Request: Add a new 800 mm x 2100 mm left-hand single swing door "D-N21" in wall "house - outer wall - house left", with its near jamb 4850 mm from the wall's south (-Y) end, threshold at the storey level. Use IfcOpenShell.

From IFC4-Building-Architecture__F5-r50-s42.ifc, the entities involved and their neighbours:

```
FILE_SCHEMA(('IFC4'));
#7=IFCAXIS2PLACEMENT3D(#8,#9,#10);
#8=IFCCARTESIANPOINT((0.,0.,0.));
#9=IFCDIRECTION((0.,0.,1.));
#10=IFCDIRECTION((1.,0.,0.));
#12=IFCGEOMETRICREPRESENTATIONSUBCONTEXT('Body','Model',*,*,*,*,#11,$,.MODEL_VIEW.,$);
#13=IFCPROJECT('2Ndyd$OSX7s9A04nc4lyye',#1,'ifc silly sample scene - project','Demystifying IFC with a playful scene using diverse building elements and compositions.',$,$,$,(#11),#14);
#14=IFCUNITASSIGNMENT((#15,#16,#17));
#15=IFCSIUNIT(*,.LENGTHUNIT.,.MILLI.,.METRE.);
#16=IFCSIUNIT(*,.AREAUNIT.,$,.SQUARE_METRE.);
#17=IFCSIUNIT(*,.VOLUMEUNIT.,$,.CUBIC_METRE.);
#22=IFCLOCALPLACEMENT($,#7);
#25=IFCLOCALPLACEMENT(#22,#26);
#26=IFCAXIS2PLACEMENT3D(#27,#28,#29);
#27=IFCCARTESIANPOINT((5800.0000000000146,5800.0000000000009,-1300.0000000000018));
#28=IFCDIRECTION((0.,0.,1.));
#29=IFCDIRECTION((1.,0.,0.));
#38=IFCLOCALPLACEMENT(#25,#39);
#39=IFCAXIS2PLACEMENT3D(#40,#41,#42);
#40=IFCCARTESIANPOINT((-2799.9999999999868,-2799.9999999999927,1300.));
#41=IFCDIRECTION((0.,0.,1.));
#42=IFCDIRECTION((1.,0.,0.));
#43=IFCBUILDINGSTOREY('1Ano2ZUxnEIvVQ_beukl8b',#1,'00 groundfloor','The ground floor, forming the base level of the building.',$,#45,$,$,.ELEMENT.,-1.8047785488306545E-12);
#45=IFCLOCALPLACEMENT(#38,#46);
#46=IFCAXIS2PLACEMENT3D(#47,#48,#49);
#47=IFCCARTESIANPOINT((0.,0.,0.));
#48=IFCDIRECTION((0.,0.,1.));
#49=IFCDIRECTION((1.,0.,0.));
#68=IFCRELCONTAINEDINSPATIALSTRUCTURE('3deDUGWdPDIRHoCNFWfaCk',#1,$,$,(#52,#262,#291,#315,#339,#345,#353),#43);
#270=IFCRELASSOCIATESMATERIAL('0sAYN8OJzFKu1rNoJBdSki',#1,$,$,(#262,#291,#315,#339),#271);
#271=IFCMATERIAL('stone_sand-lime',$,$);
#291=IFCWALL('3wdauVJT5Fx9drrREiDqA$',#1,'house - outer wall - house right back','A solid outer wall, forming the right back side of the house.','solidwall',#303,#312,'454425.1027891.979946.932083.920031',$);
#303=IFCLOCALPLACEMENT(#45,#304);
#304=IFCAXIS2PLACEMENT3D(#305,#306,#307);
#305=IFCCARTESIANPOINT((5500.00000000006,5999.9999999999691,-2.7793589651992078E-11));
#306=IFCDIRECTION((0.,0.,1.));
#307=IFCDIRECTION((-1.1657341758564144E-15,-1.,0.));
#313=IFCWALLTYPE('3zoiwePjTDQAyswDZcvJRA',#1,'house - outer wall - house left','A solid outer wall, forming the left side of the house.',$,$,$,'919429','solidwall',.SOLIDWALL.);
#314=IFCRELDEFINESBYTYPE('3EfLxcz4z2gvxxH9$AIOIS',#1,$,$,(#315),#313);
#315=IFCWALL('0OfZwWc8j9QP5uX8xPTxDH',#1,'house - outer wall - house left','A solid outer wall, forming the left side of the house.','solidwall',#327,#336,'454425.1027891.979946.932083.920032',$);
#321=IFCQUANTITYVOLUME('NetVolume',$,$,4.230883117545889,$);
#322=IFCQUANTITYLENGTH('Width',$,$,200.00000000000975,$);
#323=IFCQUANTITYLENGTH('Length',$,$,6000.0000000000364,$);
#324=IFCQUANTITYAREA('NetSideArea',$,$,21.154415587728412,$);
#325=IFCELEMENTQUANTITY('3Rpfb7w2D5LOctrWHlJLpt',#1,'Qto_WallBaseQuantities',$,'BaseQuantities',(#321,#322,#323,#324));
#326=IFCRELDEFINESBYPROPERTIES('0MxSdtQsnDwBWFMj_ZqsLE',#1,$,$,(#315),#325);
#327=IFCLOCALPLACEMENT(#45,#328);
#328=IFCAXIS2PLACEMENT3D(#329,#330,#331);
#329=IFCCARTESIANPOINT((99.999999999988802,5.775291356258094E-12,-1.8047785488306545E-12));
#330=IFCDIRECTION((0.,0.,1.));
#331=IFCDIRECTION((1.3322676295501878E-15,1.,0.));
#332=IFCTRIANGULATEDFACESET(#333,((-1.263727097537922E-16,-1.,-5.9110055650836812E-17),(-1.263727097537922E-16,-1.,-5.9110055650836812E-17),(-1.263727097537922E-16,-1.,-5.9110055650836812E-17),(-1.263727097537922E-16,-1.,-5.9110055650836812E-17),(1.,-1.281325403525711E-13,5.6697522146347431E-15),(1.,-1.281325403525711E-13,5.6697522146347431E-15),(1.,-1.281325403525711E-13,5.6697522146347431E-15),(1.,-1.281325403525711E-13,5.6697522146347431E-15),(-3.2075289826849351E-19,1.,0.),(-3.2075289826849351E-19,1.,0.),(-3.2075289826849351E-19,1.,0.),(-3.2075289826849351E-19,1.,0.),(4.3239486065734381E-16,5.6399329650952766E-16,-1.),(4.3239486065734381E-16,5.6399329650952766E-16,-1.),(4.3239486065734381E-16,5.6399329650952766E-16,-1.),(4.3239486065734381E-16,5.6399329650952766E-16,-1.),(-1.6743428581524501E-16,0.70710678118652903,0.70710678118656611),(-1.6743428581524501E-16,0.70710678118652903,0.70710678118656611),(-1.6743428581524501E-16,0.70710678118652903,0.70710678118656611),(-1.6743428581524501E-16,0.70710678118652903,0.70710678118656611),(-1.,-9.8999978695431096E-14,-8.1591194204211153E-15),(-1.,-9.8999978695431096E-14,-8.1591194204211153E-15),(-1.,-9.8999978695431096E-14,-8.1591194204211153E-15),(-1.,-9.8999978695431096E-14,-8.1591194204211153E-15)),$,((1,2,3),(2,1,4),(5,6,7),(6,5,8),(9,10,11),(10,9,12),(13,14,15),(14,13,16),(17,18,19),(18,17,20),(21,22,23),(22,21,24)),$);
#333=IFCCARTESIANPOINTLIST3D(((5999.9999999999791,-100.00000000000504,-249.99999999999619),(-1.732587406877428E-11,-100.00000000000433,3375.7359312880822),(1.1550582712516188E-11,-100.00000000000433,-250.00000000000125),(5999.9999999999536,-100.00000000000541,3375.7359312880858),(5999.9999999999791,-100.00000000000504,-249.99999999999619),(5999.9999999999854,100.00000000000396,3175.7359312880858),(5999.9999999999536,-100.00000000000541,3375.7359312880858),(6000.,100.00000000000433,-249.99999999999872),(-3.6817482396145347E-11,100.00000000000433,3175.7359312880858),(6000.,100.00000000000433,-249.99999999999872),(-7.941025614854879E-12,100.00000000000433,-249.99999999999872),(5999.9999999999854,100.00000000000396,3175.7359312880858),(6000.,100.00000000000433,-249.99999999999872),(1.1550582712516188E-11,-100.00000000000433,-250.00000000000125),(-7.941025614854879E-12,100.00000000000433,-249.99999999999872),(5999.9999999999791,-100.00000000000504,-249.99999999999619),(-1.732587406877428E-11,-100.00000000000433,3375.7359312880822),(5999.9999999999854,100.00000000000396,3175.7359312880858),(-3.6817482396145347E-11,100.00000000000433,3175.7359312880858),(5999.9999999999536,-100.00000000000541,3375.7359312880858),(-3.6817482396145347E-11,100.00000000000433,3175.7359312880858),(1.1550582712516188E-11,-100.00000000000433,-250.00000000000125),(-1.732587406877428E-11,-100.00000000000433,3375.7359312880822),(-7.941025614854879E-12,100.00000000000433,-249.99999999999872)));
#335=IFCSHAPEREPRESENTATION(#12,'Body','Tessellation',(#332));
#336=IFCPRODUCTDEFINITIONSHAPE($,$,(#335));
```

```python
import numpy as np
import ifcopenshell
import ifcopenshell.api.feature
import ifcopenshell.api.geometry
import ifcopenshell.api.pset
import ifcopenshell.api.root
import ifcopenshell.api.spatial
import ifcopenshell.geom
import ifcopenshell.util.element
import ifcopenshell.util.placement
import ifcopenshell.util.representation
import ifcopenshell.util.shape
import ifcopenshell.util.unit

model = ifcopenshell.open("IFC4-Building-Architecture__F5-r50-s42.ifc")
unit_scale = ifcopenshell.util.unit.calculate_unit_scale(model)
area_scale = ifcopenshell.util.unit.calculate_unit_scale(model, "AREAUNIT")
volume_scale = ifcopenshell.util.unit.calculate_unit_scale(model, "VOLUMEUNIT")
settings = ifcopenshell.geom.settings()


def volume(element):
    """Net volume in cubic metres, openings subtracted."""
    shape = ifcopenshell.geom.create_shape(settings, element)
    return ifcopenshell.util.shape.get_volume(shape.geometry)


wall = model.by_guid("0OfZwWc8j9QP5uX8xPTxDH")
storey = ifcopenshell.util.element.get_container(wall, ifc_class="IfcBuildingStorey")
context = ifcopenshell.util.representation.get_context(model, "Model", "Body", "MODEL_VIEW")
before = volume(wall)

width, height, from_end, sill = 0.8, 2.1, 4.85, 0.0  # metres

# The wall runs along its own X axis, and the end named is its -X end.
wall_shape = ifcopenshell.geom.create_shape(settings, wall)
x, y, z = ifcopenshell.util.shape.get_vertices(wall_shape.geometry).T
start = x.min() + from_end
face, thickness = float(y.min()), float(y.max() - y.min())
wall_matrix = ifcopenshell.util.placement.get_local_placement(wall.ObjectPlacement)
level = ifcopenshell.util.placement.get_local_placement(storey.ObjectPlacement)[2, 3]


def in_wall(x, y):
    """Placement at x, y metres in the wall's axes, at sill height."""
    matrix = wall_matrix.copy()
    matrix[:, 3] = wall_matrix @ np.array([x / unit_scale, y / unit_scale, 0.0, 1.0])
    matrix[2, 3] = level + sill / unit_scale
    return matrix


# Opening: a box that overshoots both wall faces by 50 mm.
opening = ifcopenshell.api.root.create_entity(model, ifc_class="IfcOpeningElement", predefined_type="OPENING")
box = ifcopenshell.api.geometry.add_wall_representation(
    model, context=context, length=width, height=height, thickness=thickness + 0.1
)
ifcopenshell.api.geometry.assign_representation(model, product=opening, representation=box)
ifcopenshell.api.geometry.edit_object_placement(model, product=opening, matrix=in_wall(start, face - 0.05), is_si=False)
ifcopenshell.api.feature.add_feature(model, feature=opening, element=wall)

door = ifcopenshell.api.root.create_entity(model, ifc_class="IfcDoor", name="D-N21", predefined_type="DOOR")
door.OverallWidth, door.OverallHeight = width / unit_scale, height / unit_scale
door.OperationType = "SINGLE_SWING_LEFT"
body = ifcopenshell.api.geometry.add_door_representation(
    model,
    context=context,
    overall_width=door.OverallWidth,
    overall_height=door.OverallHeight,
    operation_type="SINGLE_SWING_LEFT",
    lining_properties={"LiningDepth": thickness / unit_scale, "ThresholdDepth": thickness / unit_scale},
)
ifcopenshell.api.geometry.assign_representation(model, product=door, representation=body)
ifcopenshell.api.spatial.assign_container(model, products=[door], relating_structure=storey)
ifcopenshell.api.feature.add_filling(model, opening=opening, element=door)

# The lining spans the wall, so the door starts at the wall face.
ifcopenshell.api.geometry.edit_object_placement(model, product=door, matrix=in_wall(start, face), is_si=False)

after = volume(wall)

# Update the wall's stored quantities.
qto = model.by_id(ifcopenshell.util.element.get_pset(wall, "Qto_WallBaseQuantities", should_inherit=False)["id"])
ifcopenshell.api.pset.edit_qto(model, qto=qto, properties={
    "NetVolume": after / volume_scale,
    "NetSideArea": after / thickness / area_scale,
})

print(f"wall volume {before:.3f} -> {after:.3f} m3")

model.write("IFC4-Building-Architecture__F5-r50-s42-out.ifc")
```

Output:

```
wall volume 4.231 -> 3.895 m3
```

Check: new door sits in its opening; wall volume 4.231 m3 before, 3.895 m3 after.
